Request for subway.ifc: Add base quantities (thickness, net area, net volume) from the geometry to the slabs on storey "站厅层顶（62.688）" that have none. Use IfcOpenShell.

First a look at what the model holds.

```python
import ifcopenshell
import ifcopenshell.util.element
import ifcopenshell.util.unit

model = ifcopenshell.open("subway.ifc")
print(model.schema)
for unit_type in ("LENGTHUNIT", "AREAUNIT", "VOLUMEUNIT"):
    print(unit_type, ifcopenshell.util.unit.calculate_unit_scale(model, unit_type))
storey = next(s for s in model.by_type("IfcBuildingStorey") if s.Name == "站厅层顶（62.688）")
slabs = [e for e in ifcopenshell.util.element.get_decomposition(storey) if e.is_a("IfcSlab")]
for e in sorted(slabs, key=lambda e: e.id()):
    print(e.id(), e.is_a(), e.Name, list(ifcopenshell.util.element.get_psets(e, qtos_only=True)), sep=" | ")
```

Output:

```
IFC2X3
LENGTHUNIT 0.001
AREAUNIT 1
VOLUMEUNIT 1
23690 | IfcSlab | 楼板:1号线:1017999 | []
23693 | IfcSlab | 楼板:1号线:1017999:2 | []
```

```python
import ifcopenshell
import ifcopenshell.api.pset
import ifcopenshell.geom
import ifcopenshell.util.element
import ifcopenshell.util.shape
import ifcopenshell.util.unit

model = ifcopenshell.open("subway.ifc")
unit_scale = ifcopenshell.util.unit.calculate_unit_scale(model)
area_scale = ifcopenshell.util.unit.calculate_unit_scale(model, "AREAUNIT")
volume_scale = ifcopenshell.util.unit.calculate_unit_scale(model, "VOLUMEUNIT")
settings = ifcopenshell.geom.settings()

storey = next(s for s in model.by_type("IfcBuildingStorey") if s.Name == "站厅层顶（62.688）")
slabs = [e for e in ifcopenshell.util.element.get_decomposition(storey) if e.is_a("IfcSlab")]

for e in sorted(slabs, key=lambda e: e.id()):
    if ifcopenshell.util.element.get_psets(e, qtos_only=True, should_inherit=False):
        continue
    # Geometry comes back in metres, in the element's own axes.
    shape = ifcopenshell.geom.create_shape(settings, e)
    values = {
        "Width": ifcopenshell.util.shape.get_z(shape.geometry) / unit_scale,
        "NetArea": ifcopenshell.util.shape.get_footprint_area(shape.geometry) / area_scale,
        "NetVolume": ifcopenshell.util.shape.get_volume(shape.geometry) / volume_scale,
    }
    qto = ifcopenshell.api.pset.add_qto(model, product=e, name="BaseQuantities")
    ifcopenshell.api.pset.edit_qto(model, qto=qto, properties=values)
    print(e.id(), {k: round(v, 3) for k, v in values.items()})

model.write("subway_rev.ifc")
```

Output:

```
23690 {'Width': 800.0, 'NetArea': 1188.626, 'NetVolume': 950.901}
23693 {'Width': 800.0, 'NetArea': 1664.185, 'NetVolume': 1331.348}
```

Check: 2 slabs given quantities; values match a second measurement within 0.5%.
